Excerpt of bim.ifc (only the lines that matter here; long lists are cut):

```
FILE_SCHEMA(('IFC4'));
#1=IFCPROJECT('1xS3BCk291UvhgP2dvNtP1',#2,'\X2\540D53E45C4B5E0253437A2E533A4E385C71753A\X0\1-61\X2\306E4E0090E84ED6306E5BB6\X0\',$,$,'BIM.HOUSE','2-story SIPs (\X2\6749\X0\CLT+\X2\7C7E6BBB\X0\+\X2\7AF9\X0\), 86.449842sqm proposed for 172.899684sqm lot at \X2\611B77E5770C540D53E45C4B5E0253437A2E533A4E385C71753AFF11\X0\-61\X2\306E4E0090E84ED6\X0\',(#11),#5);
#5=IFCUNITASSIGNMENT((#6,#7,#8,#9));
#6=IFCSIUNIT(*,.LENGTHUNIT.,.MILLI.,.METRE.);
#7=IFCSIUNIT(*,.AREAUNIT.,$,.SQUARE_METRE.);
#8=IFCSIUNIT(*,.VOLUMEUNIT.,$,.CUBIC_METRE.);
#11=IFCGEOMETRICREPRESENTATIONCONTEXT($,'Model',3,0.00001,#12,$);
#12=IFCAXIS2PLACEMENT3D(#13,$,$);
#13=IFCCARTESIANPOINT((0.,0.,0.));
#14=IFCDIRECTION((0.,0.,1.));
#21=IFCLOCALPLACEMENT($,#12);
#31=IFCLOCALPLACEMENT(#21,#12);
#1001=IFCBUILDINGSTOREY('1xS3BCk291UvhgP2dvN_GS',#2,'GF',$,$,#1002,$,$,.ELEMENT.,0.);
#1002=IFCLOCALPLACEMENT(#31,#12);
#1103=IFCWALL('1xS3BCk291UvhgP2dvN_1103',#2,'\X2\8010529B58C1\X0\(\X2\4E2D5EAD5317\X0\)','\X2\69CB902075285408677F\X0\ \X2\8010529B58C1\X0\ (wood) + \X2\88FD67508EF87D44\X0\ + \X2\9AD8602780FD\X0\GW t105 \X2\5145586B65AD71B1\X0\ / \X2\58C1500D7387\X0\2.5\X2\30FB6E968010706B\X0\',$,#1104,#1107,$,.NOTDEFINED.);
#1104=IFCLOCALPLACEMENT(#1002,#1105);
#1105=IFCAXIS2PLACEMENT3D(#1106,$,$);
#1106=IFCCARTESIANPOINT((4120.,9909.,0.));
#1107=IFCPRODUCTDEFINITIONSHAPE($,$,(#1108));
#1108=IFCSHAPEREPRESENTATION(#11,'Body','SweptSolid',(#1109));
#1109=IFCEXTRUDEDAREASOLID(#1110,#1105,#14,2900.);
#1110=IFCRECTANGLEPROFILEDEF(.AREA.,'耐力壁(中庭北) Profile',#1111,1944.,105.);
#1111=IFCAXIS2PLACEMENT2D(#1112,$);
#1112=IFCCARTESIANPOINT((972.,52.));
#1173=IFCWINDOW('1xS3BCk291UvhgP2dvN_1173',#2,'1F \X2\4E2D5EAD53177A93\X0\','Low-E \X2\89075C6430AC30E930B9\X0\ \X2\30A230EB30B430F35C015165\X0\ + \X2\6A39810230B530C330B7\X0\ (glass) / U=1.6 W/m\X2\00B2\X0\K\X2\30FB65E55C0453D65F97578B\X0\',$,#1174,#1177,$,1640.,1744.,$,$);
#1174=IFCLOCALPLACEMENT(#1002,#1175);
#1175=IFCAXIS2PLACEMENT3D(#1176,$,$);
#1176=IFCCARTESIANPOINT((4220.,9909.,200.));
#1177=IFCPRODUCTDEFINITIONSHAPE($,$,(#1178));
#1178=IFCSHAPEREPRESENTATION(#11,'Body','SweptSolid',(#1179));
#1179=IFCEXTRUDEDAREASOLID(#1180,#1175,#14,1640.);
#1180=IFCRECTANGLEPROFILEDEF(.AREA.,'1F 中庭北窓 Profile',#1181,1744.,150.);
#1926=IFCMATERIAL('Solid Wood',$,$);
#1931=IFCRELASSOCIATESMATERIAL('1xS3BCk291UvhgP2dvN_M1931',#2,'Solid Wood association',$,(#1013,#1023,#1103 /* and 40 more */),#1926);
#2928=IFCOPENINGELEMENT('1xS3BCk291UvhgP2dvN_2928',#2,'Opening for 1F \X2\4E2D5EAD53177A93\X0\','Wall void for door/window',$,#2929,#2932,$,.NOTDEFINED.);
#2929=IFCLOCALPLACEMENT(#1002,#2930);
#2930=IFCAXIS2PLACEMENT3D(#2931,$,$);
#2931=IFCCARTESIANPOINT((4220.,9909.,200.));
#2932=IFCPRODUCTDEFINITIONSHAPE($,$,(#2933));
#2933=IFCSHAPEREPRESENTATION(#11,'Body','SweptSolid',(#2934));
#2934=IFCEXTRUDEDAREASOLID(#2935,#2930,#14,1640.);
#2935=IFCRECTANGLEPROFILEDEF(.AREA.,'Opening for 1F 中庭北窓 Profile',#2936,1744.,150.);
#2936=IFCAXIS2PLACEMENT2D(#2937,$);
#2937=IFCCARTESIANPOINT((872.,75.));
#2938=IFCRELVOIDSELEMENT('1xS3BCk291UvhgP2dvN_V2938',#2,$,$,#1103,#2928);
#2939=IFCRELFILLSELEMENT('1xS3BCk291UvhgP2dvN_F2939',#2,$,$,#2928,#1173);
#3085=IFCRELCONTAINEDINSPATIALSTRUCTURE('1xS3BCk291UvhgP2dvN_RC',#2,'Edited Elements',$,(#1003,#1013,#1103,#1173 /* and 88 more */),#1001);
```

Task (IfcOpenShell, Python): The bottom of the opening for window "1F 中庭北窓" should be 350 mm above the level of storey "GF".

```python
import numpy as np
import ifcopenshell
import ifcopenshell.api.geometry
import ifcopenshell.geom
import ifcopenshell.util.element
import ifcopenshell.util.placement
import ifcopenshell.util.shape
import ifcopenshell.util.unit

model = ifcopenshell.open("bim.ifc")
unit_scale = ifcopenshell.util.unit.calculate_unit_scale(model)

window = model.by_guid("1xS3BCk291UvhgP2dvN_1173")
opening = window.FillsVoids[0].RelatingOpeningElement
storey = ifcopenshell.util.element.get_container(window, ifc_class="IfcBuildingStorey")
level = ifcopenshell.util.placement.get_local_placement(storey.ObjectPlacement)[2, 3]

# The opening's origin need not be at the sill, so measure its lowest point.
shape = ifcopenshell.geom.create_shape(ifcopenshell.geom.settings(), opening)
bottom = ifcopenshell.util.shape.get_shape_bottom_elevation(shape, shape.geometry) / unit_scale
dz = level + 350.0 - bottom

shift = np.array([0.0, 0.0, dz])
# The window is not placed relative to its opening, so move both.
for product in (opening, window):
    matrix = ifcopenshell.util.placement.get_local_placement(product.ObjectPlacement)
    matrix[:3, 3] += shift
    ifcopenshell.api.geometry.edit_object_placement(model, product=product, matrix=matrix, is_si=False)

print(f"moved by {dz * unit_scale:+.3f} m")

model.write("bim_updated.ifc")
```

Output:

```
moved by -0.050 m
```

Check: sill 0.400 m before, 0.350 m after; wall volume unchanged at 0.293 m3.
